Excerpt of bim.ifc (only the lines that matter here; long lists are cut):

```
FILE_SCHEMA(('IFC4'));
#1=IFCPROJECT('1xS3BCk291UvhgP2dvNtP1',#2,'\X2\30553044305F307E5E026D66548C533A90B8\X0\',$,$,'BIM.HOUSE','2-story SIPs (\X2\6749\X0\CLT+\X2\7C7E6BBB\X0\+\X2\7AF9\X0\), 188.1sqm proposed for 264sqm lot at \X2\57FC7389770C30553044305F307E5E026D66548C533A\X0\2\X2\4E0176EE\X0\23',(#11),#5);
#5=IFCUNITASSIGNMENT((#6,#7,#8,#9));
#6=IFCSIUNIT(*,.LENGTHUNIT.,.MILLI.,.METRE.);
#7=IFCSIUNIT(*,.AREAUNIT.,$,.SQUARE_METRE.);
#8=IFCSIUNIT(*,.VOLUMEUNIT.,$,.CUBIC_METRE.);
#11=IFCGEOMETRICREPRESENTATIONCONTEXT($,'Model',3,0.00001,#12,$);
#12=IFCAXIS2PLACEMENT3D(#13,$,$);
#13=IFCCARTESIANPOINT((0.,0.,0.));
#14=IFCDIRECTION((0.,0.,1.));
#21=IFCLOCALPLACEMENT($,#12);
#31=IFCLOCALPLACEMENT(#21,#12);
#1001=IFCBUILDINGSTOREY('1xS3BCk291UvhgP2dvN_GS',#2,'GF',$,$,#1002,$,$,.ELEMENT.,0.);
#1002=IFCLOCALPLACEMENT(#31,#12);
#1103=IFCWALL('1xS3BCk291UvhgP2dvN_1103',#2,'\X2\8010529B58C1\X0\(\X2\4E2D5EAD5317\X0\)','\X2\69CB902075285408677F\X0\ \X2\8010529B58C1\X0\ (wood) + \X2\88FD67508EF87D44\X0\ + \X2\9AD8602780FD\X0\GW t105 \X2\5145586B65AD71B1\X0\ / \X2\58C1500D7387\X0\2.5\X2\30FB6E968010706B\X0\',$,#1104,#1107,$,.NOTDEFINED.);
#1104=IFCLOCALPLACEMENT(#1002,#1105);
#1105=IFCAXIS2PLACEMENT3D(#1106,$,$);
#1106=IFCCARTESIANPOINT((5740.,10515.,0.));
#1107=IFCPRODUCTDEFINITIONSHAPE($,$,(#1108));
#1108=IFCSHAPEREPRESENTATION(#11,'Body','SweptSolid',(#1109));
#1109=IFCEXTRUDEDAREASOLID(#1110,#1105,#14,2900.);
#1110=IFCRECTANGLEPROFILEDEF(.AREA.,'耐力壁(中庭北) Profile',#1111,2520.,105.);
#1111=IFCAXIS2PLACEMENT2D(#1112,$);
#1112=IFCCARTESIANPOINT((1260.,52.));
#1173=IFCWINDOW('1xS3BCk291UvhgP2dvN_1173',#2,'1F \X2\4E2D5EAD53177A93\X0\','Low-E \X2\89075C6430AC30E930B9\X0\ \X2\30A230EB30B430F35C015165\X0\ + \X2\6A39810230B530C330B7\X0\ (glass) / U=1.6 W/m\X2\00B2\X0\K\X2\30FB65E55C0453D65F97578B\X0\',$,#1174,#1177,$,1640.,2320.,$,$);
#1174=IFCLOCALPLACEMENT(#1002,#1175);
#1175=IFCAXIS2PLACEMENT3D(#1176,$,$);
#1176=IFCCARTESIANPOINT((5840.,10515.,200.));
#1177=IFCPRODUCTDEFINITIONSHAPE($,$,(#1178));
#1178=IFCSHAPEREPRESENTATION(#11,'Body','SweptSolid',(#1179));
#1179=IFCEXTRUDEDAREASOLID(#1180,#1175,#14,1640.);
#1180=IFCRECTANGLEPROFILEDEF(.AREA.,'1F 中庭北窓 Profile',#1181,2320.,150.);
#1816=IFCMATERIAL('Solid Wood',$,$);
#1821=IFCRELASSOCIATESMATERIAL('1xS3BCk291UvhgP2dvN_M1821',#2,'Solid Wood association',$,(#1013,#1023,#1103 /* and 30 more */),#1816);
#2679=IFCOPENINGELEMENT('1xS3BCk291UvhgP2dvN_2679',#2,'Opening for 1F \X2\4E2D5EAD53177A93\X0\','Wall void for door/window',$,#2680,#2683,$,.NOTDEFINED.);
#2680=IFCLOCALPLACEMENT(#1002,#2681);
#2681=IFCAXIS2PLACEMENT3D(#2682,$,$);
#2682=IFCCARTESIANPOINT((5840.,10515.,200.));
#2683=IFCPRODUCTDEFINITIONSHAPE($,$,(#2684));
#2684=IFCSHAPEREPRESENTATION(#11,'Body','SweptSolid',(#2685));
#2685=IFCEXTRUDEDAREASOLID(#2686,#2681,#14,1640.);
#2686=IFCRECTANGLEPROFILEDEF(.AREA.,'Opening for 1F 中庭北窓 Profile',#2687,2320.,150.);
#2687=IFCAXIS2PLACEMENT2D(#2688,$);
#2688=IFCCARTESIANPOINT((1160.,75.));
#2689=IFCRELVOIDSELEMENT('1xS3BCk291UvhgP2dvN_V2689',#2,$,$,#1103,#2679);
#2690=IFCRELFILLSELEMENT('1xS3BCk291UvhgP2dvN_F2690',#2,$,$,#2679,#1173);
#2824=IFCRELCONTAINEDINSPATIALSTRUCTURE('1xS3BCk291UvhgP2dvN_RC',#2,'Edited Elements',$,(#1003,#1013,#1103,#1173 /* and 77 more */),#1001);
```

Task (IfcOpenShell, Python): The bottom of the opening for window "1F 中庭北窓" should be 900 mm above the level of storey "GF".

```python
import numpy as np
import ifcopenshell
import ifcopenshell.api.geometry
import ifcopenshell.geom
import ifcopenshell.util.element
import ifcopenshell.util.placement
import ifcopenshell.util.shape
import ifcopenshell.util.unit

model = ifcopenshell.open("bim.ifc")
unit_scale = ifcopenshell.util.unit.calculate_unit_scale(model)

window = model.by_guid("1xS3BCk291UvhgP2dvN_1173")
opening = window.FillsVoids[0].RelatingOpeningElement
storey = ifcopenshell.util.element.get_container(window, ifc_class="IfcBuildingStorey")
level = ifcopenshell.util.placement.get_local_placement(storey.ObjectPlacement)[2, 3]

# The opening's origin need not be at the sill, so measure its lowest point.
shape = ifcopenshell.geom.create_shape(ifcopenshell.geom.settings(), opening)
bottom = ifcopenshell.util.shape.get_shape_bottom_elevation(shape, shape.geometry) / unit_scale
dz = level + 900.0 - bottom

shift = np.array([0.0, 0.0, dz])
# The window is not placed relative to its opening, so move both.
for product in (opening, window):
    matrix = ifcopenshell.util.placement.get_local_placement(product.ObjectPlacement)
    matrix[:3, 3] += shift
    ifcopenshell.api.geometry.edit_object_placement(model, product=product, matrix=matrix, is_si=False)

print(f"moved by {dz * unit_scale:+.3f} m")

model.write("bim_rev.ifc")
```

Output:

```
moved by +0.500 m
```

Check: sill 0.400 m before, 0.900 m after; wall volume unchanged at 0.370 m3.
